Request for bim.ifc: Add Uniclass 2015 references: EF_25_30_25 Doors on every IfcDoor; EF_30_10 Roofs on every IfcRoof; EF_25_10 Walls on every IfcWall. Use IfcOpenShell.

First a look at what the model holds.

```python
import ifcopenshell

model = ifcopenshell.open("bim.ifc")
print(model.schema)
print("classifications:", [c.Name for c in model.by_type("IfcClassification")])
for ifc_class in ("IfcDoor", "IfcRoof", "IfcStair", "IfcWall", "IfcWindow"):
    print(ifc_class, len(model.by_type(ifc_class)))
```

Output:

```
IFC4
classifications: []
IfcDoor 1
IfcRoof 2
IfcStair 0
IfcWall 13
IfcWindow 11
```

```python
import ifcopenshell
import ifcopenshell.api.classification

model = ifcopenshell.open("bim.ifc")

system = ifcopenshell.api.classification.add_classification(model, classification="Uniclass 2015")

codes = {
    "IfcDoor": ("EF_25_30_25", "Doors"),
    "IfcRoof": ("EF_30_10", "Roofs"),
    "IfcWall": ("EF_25_10", "Walls"),
}
for ifc_class, (code, name) in codes.items():
    products = model.by_type(ifc_class)
    ifcopenshell.api.classification.add_reference(
        model, products=products, classification=system, identification=code, name=name
    )
    print(code, len(products))

model.write("bim_v2.ifc")
```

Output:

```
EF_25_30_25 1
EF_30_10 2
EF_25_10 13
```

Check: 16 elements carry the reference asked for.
